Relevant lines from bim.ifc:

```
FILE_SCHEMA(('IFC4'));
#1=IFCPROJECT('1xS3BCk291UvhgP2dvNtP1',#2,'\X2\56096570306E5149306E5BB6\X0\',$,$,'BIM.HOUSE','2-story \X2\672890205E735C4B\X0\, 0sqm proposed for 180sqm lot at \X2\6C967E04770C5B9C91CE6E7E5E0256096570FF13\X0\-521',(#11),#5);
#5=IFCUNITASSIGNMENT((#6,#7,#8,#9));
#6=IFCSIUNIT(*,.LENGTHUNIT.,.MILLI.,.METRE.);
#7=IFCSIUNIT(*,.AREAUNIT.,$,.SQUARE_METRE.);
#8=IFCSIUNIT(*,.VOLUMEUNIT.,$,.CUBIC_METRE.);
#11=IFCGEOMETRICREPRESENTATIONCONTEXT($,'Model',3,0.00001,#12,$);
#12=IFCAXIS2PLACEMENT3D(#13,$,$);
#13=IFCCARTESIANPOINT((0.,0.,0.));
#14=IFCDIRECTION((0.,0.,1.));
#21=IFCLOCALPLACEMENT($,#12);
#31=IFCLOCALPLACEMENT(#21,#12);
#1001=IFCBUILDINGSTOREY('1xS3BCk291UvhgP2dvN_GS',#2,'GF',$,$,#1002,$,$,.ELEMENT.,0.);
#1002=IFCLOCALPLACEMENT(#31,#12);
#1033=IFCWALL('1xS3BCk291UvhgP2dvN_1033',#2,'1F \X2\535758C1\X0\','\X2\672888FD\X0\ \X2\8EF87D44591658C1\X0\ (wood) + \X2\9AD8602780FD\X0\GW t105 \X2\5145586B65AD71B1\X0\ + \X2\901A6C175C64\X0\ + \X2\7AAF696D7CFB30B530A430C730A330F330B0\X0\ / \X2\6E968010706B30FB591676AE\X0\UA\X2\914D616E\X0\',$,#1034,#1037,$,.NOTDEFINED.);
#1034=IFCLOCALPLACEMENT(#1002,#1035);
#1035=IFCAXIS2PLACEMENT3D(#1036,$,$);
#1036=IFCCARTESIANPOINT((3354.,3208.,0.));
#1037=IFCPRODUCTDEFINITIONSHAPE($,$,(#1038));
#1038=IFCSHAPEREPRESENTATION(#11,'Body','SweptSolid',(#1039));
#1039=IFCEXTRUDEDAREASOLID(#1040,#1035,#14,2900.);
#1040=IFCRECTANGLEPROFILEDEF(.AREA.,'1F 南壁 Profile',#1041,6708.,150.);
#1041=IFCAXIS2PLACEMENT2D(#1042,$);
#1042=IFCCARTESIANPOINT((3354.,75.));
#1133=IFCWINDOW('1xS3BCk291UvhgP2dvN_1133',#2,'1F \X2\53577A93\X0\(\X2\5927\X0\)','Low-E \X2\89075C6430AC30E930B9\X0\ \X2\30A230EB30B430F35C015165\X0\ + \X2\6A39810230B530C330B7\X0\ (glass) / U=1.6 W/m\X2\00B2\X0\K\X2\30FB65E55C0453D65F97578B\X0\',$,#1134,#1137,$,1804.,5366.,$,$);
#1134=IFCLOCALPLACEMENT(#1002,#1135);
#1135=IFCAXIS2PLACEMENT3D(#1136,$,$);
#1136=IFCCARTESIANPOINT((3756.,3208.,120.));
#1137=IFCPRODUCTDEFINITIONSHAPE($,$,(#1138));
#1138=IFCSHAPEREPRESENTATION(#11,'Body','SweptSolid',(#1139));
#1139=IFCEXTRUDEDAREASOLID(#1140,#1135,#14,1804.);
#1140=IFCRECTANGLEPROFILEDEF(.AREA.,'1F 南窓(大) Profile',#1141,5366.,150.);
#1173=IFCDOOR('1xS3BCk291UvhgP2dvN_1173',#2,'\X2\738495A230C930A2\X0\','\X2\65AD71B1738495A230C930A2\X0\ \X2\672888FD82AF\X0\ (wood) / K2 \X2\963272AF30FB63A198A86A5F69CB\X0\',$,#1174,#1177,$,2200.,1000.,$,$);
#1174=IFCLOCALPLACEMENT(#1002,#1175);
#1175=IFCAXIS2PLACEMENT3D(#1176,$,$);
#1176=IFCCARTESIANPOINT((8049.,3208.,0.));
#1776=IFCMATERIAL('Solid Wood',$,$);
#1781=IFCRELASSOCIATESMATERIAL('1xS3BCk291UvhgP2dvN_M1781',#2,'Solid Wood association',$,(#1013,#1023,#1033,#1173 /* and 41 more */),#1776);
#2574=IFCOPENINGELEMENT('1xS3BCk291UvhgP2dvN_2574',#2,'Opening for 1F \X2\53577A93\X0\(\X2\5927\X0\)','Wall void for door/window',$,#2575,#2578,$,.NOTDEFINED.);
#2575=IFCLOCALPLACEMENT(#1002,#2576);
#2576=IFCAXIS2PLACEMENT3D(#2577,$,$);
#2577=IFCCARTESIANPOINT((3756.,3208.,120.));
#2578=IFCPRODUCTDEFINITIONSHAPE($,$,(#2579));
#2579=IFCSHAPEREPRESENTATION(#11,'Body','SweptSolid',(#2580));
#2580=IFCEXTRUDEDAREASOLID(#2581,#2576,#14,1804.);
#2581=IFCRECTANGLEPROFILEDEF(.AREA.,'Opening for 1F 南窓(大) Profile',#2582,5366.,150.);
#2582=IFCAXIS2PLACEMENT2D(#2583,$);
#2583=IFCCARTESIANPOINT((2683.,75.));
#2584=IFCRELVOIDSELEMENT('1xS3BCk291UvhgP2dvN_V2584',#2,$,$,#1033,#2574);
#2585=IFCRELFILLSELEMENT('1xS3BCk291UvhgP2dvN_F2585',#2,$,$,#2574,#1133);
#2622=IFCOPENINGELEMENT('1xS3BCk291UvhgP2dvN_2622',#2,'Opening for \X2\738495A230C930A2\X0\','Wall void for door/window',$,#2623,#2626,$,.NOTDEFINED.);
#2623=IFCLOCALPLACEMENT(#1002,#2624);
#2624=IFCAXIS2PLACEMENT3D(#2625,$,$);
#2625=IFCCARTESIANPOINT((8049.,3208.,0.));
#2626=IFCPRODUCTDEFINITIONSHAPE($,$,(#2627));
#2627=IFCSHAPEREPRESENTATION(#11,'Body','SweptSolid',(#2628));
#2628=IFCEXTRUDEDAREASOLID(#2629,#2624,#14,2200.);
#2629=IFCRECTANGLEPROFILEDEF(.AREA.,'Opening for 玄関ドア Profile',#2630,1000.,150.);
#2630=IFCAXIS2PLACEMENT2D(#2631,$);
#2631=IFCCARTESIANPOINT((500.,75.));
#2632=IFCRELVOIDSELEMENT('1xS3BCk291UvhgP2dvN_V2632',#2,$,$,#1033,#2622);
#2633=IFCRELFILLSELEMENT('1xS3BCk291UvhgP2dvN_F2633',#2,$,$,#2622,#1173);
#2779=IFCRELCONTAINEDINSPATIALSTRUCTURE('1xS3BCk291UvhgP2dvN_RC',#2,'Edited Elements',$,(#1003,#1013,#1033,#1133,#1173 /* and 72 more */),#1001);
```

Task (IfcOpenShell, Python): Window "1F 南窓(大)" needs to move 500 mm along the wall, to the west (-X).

```python
import ifcopenshell
import ifcopenshell.api.geometry
import ifcopenshell.util.placement

model = ifcopenshell.open("bim.ifc")

window = model.by_guid("1xS3BCk291UvhgP2dvN_1133")
opening = window.FillsVoids[0].RelatingOpeningElement
wall = opening.VoidsElements[0].RelatingBuildingElement

wall_matrix = ifcopenshell.util.placement.get_local_placement(wall.ObjectPlacement)
shift = wall_matrix[:3, 0] * -500.0
before = ifcopenshell.util.placement.get_local_placement(window.ObjectPlacement)[:3, 3].copy()

# The window is not placed relative to its opening, so move both.
for product in (opening, window):
    matrix = ifcopenshell.util.placement.get_local_placement(product.ObjectPlacement)
    matrix[:3, 3] += shift
    ifcopenshell.api.geometry.edit_object_placement(model, product=product, matrix=matrix, is_si=False)

after = ifcopenshell.util.placement.get_local_placement(window.ObjectPlacement)[:3, 3]
print("window moved by", (after - before).round(3) + 0.0)

model.write("bim_updated.ifc")
```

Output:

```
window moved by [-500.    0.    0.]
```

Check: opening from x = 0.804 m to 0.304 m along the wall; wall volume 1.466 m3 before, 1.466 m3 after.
